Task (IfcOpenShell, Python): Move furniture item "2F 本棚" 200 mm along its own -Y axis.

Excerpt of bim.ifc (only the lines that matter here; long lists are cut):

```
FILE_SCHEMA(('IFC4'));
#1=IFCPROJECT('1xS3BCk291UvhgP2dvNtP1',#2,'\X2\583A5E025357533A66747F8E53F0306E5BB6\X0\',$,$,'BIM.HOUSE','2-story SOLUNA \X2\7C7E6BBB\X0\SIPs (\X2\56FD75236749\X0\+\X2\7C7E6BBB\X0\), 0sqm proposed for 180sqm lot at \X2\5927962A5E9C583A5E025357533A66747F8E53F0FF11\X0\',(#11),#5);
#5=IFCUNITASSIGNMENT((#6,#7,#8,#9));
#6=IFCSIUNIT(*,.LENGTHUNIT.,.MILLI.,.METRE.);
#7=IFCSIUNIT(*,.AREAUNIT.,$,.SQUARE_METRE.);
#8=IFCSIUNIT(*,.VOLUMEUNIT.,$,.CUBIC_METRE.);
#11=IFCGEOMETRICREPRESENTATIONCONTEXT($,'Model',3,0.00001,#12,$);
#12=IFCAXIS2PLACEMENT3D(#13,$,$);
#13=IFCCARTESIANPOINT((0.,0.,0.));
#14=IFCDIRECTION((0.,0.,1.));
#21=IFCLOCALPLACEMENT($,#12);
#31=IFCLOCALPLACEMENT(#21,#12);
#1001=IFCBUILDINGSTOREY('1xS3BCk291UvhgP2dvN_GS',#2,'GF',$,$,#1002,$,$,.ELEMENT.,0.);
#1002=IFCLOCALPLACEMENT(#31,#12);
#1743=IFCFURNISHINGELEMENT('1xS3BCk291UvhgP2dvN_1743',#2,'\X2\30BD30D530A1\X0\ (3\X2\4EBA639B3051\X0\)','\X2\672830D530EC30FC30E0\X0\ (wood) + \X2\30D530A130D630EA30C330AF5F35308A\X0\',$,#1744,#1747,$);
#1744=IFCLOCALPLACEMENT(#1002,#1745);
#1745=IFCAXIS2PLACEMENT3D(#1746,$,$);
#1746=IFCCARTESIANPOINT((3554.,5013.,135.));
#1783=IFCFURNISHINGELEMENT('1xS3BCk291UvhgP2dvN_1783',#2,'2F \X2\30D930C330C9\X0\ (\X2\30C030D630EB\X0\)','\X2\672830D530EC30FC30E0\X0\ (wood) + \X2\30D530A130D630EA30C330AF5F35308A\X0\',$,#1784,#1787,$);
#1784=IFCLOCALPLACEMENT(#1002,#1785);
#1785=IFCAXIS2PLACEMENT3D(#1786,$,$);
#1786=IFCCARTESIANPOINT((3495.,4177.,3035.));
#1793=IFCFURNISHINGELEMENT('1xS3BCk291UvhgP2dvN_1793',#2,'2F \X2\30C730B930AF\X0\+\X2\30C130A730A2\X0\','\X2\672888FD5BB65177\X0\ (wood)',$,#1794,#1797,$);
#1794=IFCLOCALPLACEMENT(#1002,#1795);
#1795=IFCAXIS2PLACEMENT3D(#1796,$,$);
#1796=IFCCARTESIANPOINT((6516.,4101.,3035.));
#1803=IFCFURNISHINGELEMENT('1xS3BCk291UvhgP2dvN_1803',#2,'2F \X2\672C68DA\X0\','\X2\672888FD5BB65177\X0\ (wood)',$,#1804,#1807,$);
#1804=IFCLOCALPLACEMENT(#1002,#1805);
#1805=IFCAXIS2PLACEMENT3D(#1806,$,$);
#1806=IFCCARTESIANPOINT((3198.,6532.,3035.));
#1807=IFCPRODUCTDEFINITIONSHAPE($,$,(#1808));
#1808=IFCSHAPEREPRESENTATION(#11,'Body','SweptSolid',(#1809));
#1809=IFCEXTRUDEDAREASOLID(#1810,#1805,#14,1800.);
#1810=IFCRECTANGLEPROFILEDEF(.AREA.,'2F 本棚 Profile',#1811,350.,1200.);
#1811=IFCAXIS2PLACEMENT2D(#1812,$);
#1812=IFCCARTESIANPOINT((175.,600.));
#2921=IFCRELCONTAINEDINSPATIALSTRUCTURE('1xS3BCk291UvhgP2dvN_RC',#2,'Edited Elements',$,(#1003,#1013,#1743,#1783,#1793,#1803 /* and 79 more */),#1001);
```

```python
import ifcopenshell
import ifcopenshell.api.geometry
import ifcopenshell.util.placement

model = ifcopenshell.open("bim.ifc")

item = model.by_id(1803)
matrix = ifcopenshell.util.placement.get_local_placement(item.ObjectPlacement)
matrix[:3, 3] -= matrix[:3, 1] * 200.0
ifcopenshell.api.geometry.edit_object_placement(model, product=item, matrix=matrix, is_si=False)

print(ifcopenshell.util.placement.get_local_placement(item.ObjectPlacement).round(3) + 0.0)

model.write("bim_rev.ifc")
```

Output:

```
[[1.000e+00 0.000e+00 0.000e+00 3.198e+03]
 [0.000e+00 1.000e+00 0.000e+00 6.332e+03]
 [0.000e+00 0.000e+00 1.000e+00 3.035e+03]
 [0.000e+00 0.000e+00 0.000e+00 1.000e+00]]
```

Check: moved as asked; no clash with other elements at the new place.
